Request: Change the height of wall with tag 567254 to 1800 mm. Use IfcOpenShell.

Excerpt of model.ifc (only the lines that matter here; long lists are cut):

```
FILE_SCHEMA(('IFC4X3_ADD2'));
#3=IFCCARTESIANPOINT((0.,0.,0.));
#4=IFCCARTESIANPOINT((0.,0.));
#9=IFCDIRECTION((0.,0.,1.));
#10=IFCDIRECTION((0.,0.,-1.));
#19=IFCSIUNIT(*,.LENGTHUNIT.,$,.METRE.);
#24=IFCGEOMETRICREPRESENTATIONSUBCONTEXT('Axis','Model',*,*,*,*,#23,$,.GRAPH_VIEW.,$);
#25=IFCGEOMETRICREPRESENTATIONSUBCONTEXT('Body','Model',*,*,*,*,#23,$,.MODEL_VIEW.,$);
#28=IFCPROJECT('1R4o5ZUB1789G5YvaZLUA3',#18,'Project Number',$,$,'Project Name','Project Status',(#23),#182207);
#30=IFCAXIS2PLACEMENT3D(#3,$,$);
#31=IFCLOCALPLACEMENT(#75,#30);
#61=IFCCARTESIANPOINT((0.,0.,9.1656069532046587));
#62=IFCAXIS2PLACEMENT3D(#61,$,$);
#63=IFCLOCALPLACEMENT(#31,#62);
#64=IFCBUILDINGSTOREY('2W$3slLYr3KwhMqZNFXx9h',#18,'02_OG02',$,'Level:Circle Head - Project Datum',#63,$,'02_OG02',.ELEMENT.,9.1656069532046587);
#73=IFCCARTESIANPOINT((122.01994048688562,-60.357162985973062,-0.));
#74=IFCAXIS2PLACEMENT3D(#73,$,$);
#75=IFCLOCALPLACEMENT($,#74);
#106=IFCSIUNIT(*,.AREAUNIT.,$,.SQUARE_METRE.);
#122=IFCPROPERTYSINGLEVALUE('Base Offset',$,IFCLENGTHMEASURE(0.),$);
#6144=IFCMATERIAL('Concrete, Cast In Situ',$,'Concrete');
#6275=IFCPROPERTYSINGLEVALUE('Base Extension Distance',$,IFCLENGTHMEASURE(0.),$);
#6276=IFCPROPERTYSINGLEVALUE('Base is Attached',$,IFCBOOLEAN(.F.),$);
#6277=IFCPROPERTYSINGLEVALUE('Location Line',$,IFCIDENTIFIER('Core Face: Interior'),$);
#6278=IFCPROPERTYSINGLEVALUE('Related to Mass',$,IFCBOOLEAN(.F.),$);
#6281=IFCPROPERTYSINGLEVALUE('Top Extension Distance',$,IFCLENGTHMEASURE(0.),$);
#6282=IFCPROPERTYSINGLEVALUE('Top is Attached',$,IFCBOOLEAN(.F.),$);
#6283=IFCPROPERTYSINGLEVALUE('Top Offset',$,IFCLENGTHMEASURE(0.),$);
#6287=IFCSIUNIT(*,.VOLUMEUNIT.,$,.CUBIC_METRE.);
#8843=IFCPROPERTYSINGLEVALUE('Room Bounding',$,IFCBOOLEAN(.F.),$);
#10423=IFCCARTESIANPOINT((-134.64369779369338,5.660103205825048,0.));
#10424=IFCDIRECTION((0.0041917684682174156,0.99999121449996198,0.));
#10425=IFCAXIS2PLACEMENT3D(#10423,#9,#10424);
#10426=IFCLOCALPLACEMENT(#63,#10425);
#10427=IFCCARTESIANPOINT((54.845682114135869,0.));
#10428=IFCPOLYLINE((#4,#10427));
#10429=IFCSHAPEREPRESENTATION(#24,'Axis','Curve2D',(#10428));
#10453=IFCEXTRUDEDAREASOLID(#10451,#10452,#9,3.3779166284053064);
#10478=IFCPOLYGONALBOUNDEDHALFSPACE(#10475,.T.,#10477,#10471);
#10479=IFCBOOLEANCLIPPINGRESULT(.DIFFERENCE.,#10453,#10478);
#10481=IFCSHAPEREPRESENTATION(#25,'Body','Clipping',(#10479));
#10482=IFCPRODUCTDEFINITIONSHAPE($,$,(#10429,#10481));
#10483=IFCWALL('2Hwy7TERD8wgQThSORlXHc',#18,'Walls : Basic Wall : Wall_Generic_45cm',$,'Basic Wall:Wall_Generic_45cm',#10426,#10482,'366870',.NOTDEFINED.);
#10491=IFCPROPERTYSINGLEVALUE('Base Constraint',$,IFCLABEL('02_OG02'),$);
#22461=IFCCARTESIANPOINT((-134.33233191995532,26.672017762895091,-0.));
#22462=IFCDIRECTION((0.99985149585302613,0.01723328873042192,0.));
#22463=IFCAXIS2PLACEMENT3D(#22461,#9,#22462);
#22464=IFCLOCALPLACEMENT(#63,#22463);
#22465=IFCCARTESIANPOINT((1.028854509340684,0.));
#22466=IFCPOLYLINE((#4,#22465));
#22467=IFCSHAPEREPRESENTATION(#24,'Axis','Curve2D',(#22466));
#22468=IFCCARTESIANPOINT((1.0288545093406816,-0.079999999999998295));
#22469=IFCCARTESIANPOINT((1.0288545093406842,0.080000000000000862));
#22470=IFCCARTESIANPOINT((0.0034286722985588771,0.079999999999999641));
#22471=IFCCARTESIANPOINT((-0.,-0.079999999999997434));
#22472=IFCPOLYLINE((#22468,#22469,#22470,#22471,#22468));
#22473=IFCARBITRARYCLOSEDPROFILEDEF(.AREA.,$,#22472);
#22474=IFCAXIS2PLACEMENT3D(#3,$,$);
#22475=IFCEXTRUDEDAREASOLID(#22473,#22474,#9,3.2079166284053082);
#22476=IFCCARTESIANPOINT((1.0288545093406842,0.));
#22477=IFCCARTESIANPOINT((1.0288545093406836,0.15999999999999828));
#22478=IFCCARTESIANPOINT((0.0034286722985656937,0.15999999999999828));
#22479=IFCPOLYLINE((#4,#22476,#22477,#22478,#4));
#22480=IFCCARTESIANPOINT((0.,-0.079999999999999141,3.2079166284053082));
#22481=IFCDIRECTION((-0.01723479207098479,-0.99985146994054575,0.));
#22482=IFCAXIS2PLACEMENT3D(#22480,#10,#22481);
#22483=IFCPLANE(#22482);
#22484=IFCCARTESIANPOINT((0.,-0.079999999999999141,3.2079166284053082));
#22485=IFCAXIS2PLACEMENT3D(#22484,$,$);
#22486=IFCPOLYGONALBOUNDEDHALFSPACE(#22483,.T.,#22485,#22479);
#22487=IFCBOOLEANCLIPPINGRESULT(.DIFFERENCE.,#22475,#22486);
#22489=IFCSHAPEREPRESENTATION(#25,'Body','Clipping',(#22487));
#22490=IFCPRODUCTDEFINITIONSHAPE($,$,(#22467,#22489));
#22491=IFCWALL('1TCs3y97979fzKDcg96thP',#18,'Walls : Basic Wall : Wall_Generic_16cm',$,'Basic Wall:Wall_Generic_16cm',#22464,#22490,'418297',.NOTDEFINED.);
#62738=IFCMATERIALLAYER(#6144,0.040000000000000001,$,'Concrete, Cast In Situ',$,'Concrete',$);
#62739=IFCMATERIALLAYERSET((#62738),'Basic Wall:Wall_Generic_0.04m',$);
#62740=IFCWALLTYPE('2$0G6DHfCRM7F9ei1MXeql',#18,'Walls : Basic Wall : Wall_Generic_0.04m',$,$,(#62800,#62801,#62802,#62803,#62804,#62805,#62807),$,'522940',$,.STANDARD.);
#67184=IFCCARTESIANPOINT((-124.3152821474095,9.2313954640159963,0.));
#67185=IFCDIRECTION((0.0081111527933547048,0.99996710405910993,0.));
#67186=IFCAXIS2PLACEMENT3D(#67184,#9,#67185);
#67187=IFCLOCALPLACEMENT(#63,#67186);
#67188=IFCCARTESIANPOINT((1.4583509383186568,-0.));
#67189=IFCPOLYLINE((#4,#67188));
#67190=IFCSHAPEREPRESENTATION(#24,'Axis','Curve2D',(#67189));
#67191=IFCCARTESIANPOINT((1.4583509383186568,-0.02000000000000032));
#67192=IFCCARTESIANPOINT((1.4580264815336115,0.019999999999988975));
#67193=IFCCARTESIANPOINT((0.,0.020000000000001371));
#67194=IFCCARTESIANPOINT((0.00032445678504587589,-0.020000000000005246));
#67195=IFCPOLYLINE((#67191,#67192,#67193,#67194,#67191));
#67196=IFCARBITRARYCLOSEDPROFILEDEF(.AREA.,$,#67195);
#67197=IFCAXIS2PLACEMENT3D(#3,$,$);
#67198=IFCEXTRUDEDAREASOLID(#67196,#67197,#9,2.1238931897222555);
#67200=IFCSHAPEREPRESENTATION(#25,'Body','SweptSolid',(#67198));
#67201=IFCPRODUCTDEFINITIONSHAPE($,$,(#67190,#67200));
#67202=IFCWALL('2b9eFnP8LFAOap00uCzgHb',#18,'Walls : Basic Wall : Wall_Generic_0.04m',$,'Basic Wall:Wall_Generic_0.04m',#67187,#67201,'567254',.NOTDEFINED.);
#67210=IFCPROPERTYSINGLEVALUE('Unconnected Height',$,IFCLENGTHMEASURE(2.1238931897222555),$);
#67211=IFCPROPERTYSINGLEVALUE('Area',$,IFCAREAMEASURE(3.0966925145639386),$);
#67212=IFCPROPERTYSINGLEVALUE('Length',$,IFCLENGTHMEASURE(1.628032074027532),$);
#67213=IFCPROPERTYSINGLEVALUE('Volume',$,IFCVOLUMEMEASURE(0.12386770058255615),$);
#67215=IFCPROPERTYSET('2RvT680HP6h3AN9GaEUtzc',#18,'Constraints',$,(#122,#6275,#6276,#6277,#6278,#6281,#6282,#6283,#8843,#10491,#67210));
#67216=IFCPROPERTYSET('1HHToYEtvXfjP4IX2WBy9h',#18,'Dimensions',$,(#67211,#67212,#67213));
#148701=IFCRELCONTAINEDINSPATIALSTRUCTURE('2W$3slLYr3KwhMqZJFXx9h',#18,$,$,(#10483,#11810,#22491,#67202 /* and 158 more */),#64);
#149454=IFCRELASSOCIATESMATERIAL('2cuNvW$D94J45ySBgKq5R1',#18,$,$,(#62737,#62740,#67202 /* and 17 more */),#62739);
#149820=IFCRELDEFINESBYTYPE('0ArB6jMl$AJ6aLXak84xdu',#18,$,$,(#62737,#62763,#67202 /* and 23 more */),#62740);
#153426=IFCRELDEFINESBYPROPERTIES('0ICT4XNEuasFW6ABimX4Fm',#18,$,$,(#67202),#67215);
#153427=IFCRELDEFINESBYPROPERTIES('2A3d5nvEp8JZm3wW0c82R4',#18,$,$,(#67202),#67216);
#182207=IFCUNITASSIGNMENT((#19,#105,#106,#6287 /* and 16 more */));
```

```python
import ifcopenshell
import ifcopenshell.api.pset
import ifcopenshell.geom
import ifcopenshell.util.element
import ifcopenshell.util.representation
import ifcopenshell.util.shape
import ifcopenshell.util.unit

model = ifcopenshell.open("model.ifc")
unit_scale = ifcopenshell.util.unit.calculate_unit_scale(model)
area_scale = ifcopenshell.util.unit.calculate_unit_scale(model, "AREAUNIT")
volume_scale = ifcopenshell.util.unit.calculate_unit_scale(model, "VOLUMEUNIT")
settings = ifcopenshell.geom.settings()


def volume(element):
    """Net volume in cubic metres, openings subtracted."""
    shape = ifcopenshell.geom.create_shape(settings, element)
    return ifcopenshell.util.shape.get_volume(shape.geometry)


wall = model.by_guid("2b9eFnP8LFAOap00uCzgHb")
before = volume(wall)

body = ifcopenshell.util.representation.get_representation(wall, "Model", "Body")
solid = body.Items[0]
old_height = solid.Depth
solid.Depth = 1.8 / unit_scale
after = volume(wall)
thickness = 0.04  # wall thickness in metres

# Update the stored height, areas and volumes.
pset = model.by_id(ifcopenshell.util.element.get_pset(wall, "Constraints", should_inherit=False)["id"])
ifcopenshell.api.pset.edit_pset(model, pset=pset, properties={
    "Unconnected Height": model.create_entity("IfcLengthMeasure", solid.Depth),
})
pset = model.by_id(ifcopenshell.util.element.get_pset(wall, "Dimensions", should_inherit=False)["id"])
ifcopenshell.api.pset.edit_pset(model, pset=pset, properties={
    "Area": model.create_entity("IfcAreaMeasure", after / thickness / area_scale),
    "Volume": model.create_entity("IfcVolumeMeasure", after / volume_scale),
})

print(f"height {old_height:g} -> {solid.Depth:g}, volume {before:.3f} -> {after:.3f} m3")

model.write("model_rev.ifc")
```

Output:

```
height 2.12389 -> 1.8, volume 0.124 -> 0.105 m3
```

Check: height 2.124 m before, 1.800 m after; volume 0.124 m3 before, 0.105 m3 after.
